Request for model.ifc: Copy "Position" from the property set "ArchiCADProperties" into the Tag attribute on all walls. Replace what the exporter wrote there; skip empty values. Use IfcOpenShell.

First a look at what the model holds.

```python
import ifcopenshell
import ifcopenshell.util.element

model = ifcopenshell.open("model.ifc")
print(model.schema)
walls = model.by_type("IfcWall")
print(len(walls), "walls")
for e in walls[:8]:
    source = ifcopenshell.util.element.get_pset(e, "ArchiCADProperties", "Position")
    target = e.Tag
    print(e.id(), repr(source), repr(target), sep=" | ")
```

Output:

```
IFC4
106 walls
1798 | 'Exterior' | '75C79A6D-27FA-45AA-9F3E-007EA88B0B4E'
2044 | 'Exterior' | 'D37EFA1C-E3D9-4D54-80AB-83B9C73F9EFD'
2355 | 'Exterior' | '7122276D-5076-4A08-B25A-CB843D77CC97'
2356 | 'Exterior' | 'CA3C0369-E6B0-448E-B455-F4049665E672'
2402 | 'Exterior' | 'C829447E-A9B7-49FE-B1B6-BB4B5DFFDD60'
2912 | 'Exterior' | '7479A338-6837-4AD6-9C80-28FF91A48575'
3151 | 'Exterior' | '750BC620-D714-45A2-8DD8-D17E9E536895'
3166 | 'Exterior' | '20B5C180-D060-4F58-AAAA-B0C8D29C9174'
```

```python
import ifcopenshell
import ifcopenshell.util.element

model = ifcopenshell.open("model.ifc")

count = 0
for e in model.by_type("IfcWall"):
    value = ifcopenshell.util.element.get_pset(e, "ArchiCADProperties", "Position")
    current = e.Tag
    if not value or not value.strip() or current == value:
        continue
    e.Tag = value
    count += 1

print(count, "walls updated")

model.write("model_v2.ifc")
```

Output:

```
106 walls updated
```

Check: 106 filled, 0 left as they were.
